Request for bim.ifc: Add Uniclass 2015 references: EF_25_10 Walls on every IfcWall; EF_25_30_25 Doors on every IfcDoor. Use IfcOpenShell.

First a look at what the model holds.

```python
import ifcopenshell

model = ifcopenshell.open("bim.ifc")
print(model.schema)
print("classifications:", [c.Name for c in model.by_type("IfcClassification")])
for ifc_class in ("IfcDoor", "IfcRoof", "IfcStair", "IfcWall", "IfcWindow"):
    print(ifc_class, len(model.by_type(ifc_class)))
```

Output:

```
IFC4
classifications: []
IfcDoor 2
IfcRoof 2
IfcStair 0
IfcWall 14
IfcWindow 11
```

```python
import ifcopenshell
import ifcopenshell.api.classification

model = ifcopenshell.open("bim.ifc")

system = ifcopenshell.api.classification.add_classification(model, classification="Uniclass 2015")

codes = {
    "IfcWall": ("EF_25_10", "Walls"),
    "IfcDoor": ("EF_25_30_25", "Doors"),
}
for ifc_class, (code, name) in codes.items():
    products = model.by_type(ifc_class)
    ifcopenshell.api.classification.add_reference(
        model, products=products, classification=system, identification=code, name=name
    )
    print(code, len(products))

model.write("bim_updated.ifc")
```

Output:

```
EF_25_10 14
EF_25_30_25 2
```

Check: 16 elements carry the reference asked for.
